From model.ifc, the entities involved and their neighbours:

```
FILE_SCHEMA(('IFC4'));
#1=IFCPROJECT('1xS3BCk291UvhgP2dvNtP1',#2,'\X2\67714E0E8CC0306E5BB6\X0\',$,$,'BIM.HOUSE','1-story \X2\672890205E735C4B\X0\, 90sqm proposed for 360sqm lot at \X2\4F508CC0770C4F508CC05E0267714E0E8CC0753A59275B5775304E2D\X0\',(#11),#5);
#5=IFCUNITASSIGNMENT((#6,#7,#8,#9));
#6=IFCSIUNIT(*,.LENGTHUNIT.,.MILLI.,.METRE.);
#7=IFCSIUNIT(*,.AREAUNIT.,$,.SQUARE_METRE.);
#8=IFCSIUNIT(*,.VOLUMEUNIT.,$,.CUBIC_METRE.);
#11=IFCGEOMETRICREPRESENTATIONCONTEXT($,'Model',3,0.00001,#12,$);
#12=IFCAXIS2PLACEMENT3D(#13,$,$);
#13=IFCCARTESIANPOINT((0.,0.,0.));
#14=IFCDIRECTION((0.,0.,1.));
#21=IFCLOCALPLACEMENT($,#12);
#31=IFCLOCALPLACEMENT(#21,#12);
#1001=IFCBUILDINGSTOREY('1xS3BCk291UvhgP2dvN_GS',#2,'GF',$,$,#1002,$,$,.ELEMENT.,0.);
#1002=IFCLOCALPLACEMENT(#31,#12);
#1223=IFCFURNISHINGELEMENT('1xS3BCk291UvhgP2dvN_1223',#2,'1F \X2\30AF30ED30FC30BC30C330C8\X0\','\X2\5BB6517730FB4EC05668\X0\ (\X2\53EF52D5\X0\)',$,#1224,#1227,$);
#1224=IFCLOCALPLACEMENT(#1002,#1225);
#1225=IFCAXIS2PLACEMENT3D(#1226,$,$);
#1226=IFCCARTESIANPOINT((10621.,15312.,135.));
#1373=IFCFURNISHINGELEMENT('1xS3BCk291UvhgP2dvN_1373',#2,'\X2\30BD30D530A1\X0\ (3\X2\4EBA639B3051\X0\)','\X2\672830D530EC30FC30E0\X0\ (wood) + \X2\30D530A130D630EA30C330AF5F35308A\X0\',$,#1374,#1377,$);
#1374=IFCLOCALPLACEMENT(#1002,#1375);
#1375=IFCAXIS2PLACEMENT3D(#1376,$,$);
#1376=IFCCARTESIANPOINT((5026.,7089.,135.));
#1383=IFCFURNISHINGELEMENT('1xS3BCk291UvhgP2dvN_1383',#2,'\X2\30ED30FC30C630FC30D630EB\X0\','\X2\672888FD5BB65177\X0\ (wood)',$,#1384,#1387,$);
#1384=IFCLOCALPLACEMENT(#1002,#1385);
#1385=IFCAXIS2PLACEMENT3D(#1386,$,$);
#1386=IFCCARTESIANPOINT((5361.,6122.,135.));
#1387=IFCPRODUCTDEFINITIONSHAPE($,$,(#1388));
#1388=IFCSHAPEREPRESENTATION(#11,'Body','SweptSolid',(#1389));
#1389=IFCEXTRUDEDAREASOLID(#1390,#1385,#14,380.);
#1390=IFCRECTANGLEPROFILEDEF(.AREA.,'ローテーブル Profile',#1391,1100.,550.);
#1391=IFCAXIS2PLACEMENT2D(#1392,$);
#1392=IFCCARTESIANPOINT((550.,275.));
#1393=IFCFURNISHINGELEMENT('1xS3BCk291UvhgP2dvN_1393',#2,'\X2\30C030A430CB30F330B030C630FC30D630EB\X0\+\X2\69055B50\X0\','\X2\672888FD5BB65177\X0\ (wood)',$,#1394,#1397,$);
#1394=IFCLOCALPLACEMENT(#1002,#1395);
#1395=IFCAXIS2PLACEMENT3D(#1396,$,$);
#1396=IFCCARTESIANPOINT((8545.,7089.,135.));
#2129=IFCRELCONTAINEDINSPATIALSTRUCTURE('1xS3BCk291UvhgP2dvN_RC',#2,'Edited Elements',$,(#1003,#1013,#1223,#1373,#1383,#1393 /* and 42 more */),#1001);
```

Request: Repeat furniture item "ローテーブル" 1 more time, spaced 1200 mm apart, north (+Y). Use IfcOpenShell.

```python
import numpy as np
import ifcopenshell
import ifcopenshell.api.geometry
import ifcopenshell.api.root
import ifcopenshell.util.element
import ifcopenshell.util.placement

model = ifcopenshell.open("model.ifc")


def reuse_history(source, copy):
    """copy_class also copies each property set's owner history, people and application; keep the originals."""
    for rel in copy.IsDefinedBy:
        if rel.is_a("IfcRelDefinesByProperties") and (history := rel.RelatingPropertyDefinition.OwnerHistory):
            rel.RelatingPropertyDefinition.OwnerHistory = source.OwnerHistory
            ifcopenshell.util.element.remove_deep2(model, history)


source = model.by_id(1383)
base = ifcopenshell.util.placement.get_local_placement(source.ObjectPlacement)
step = np.array([0.0, 1.0, 0.0]) * 1200.0

for i in range(1, 2):
    copy = ifcopenshell.api.root.copy_class(model, product=source)
    copy.Representation = ifcopenshell.util.element.copy_deep(
        model, source.Representation, exclude=["IfcGeometricRepresentationContext", "IfcRepresentationMap"]
    )
    reuse_history(source, copy)
    matrix = base.copy()
    matrix[:3, 3] += i * step
    print("added at", matrix[:3, 3].round(3) + 0.0)
    ifcopenshell.api.geometry.edit_object_placement(model, product=copy, matrix=matrix, is_si=False)

model.write("model_edited.ifc")
```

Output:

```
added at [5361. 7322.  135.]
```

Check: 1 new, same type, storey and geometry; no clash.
